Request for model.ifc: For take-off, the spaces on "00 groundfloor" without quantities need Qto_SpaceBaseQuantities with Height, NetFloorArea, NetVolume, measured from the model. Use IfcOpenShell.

First a look at what the model holds.

```python
import ifcopenshell
import ifcopenshell.util.element
import ifcopenshell.util.unit

model = ifcopenshell.open("model.ifc")
print(model.schema)
for unit_type in ("LENGTHUNIT", "AREAUNIT", "VOLUMEUNIT"):
    print(unit_type, ifcopenshell.util.unit.calculate_unit_scale(model, unit_type))
storey = next(s for s in model.by_type("IfcBuildingStorey") if s.Name == "00 groundfloor")
spaces = [e for e in ifcopenshell.util.element.get_decomposition(storey) if e.is_a("IfcSpace")]
for e in sorted(spaces, key=lambda e: e.id()):
    print(e.id(), e.is_a(), e.Name, list(ifcopenshell.util.element.get_psets(e, qtos_only=True)), sep=" | ")
```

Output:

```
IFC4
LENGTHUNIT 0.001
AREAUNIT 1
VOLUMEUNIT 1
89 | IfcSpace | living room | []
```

```python
import ifcopenshell
import ifcopenshell.api.pset
import ifcopenshell.geom
import ifcopenshell.util.element
import ifcopenshell.util.shape
import ifcopenshell.util.unit

model = ifcopenshell.open("model.ifc")
unit_scale = ifcopenshell.util.unit.calculate_unit_scale(model)
area_scale = ifcopenshell.util.unit.calculate_unit_scale(model, "AREAUNIT")
volume_scale = ifcopenshell.util.unit.calculate_unit_scale(model, "VOLUMEUNIT")
settings = ifcopenshell.geom.settings()

storey = next(s for s in model.by_type("IfcBuildingStorey") if s.Name == "00 groundfloor")
spaces = [e for e in ifcopenshell.util.element.get_decomposition(storey) if e.is_a("IfcSpace")]

for e in sorted(spaces, key=lambda e: e.id()):
    if ifcopenshell.util.element.get_psets(e, qtos_only=True, should_inherit=False):
        continue
    # Geometry comes back in metres, in the element's own axes.
    shape = ifcopenshell.geom.create_shape(settings, e)
    values = {
        "Height": ifcopenshell.util.shape.get_z(shape.geometry) / unit_scale,
        "NetFloorArea": ifcopenshell.util.shape.get_footprint_area(shape.geometry) / area_scale,
        "NetVolume": ifcopenshell.util.shape.get_volume(shape.geometry) / volume_scale,
    }
    qto = ifcopenshell.api.pset.add_qto(model, product=e, name="Qto_SpaceBaseQuantities")
    ifcopenshell.api.pset.edit_qto(model, qto=qto, properties=values)
    print(e.id(), {k: round(v, 3) for k, v in values.items()})

model.write("model_updated.ifc")
```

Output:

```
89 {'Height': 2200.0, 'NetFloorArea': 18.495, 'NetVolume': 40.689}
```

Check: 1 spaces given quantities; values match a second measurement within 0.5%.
